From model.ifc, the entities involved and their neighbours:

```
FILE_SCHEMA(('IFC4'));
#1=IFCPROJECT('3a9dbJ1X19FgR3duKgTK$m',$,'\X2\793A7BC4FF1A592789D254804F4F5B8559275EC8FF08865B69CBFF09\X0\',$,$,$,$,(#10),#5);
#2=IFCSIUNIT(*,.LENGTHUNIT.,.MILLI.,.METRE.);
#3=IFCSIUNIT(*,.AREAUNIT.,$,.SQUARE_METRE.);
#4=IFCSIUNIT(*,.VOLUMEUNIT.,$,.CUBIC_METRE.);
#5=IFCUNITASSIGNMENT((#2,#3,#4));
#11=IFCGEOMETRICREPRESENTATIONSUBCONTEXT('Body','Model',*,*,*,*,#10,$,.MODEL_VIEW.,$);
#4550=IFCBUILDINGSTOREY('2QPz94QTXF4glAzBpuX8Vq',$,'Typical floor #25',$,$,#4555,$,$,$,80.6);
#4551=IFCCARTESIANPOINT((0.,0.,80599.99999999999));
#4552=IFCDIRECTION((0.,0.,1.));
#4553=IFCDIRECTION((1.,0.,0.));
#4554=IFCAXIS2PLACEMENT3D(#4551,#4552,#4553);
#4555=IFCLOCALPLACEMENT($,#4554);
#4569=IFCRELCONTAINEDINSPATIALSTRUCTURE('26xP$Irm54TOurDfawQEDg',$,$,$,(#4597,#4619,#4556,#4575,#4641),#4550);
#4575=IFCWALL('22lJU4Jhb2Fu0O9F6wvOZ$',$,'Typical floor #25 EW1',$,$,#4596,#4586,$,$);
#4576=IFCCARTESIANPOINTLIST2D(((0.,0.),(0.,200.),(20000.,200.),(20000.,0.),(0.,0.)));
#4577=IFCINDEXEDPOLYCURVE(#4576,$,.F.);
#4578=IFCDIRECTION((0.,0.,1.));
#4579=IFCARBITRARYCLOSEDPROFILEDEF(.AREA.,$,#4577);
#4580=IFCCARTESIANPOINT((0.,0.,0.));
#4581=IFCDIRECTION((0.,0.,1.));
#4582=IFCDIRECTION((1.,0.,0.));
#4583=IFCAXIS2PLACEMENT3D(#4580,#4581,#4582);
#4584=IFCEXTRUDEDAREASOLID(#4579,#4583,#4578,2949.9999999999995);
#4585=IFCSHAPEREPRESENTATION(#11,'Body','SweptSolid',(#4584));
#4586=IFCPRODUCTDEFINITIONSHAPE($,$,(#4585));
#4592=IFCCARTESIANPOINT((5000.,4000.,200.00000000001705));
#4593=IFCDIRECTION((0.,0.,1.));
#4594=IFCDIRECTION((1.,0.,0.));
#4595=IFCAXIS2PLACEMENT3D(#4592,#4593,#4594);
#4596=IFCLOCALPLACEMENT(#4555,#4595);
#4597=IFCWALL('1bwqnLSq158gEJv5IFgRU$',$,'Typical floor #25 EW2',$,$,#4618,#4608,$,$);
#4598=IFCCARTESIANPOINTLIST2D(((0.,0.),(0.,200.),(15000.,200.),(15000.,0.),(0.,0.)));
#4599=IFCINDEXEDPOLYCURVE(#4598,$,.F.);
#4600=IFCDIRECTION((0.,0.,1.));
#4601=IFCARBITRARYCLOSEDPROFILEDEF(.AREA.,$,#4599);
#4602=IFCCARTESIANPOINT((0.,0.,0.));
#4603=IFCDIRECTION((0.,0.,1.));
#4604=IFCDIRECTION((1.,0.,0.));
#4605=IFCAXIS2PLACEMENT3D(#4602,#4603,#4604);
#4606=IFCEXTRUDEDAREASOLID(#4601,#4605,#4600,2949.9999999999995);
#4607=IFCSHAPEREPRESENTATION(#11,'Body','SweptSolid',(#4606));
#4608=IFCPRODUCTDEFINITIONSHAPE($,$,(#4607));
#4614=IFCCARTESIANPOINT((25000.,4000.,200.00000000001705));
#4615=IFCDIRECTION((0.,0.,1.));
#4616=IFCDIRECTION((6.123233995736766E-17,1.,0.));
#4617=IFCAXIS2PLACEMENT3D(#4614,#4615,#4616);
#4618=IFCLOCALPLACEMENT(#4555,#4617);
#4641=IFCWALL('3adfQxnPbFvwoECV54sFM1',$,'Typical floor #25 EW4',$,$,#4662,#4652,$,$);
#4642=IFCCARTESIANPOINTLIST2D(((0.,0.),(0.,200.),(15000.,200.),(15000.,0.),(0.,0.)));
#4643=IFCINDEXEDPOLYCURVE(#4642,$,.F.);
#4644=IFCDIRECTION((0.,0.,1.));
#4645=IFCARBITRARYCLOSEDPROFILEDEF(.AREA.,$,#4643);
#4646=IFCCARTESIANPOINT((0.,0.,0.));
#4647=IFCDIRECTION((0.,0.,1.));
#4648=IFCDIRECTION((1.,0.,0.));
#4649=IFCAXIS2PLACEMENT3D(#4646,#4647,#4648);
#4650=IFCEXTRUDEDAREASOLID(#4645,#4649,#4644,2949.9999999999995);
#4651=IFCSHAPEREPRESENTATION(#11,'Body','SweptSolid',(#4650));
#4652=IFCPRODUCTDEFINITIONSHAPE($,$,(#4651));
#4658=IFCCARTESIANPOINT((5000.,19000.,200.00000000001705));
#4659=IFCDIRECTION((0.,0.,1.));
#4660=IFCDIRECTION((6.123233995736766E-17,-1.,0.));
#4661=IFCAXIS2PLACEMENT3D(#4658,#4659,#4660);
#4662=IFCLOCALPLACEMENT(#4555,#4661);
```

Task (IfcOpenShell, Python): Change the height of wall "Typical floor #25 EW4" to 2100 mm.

```python
import ifcopenshell
import ifcopenshell.geom
import ifcopenshell.util.representation
import ifcopenshell.util.shape
import ifcopenshell.util.unit

model = ifcopenshell.open("model.ifc")
unit_scale = ifcopenshell.util.unit.calculate_unit_scale(model)
settings = ifcopenshell.geom.settings()


def volume(element):
    """Net volume in cubic metres, openings subtracted."""
    shape = ifcopenshell.geom.create_shape(settings, element)
    return ifcopenshell.util.shape.get_volume(shape.geometry)


wall = model.by_guid("3adfQxnPbFvwoECV54sFM1")
before = volume(wall)

body = ifcopenshell.util.representation.get_representation(wall, "Model", "Body")
solid = body.Items[0]
old_height = solid.Depth
solid.Depth = 2.1 / unit_scale
after = volume(wall)

print(f"height {old_height:g} -> {solid.Depth:g}, volume {before:.3f} -> {after:.3f} m3")

model.write("model_v2.ifc")
```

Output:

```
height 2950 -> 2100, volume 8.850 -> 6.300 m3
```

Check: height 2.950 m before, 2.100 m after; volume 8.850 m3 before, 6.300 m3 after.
